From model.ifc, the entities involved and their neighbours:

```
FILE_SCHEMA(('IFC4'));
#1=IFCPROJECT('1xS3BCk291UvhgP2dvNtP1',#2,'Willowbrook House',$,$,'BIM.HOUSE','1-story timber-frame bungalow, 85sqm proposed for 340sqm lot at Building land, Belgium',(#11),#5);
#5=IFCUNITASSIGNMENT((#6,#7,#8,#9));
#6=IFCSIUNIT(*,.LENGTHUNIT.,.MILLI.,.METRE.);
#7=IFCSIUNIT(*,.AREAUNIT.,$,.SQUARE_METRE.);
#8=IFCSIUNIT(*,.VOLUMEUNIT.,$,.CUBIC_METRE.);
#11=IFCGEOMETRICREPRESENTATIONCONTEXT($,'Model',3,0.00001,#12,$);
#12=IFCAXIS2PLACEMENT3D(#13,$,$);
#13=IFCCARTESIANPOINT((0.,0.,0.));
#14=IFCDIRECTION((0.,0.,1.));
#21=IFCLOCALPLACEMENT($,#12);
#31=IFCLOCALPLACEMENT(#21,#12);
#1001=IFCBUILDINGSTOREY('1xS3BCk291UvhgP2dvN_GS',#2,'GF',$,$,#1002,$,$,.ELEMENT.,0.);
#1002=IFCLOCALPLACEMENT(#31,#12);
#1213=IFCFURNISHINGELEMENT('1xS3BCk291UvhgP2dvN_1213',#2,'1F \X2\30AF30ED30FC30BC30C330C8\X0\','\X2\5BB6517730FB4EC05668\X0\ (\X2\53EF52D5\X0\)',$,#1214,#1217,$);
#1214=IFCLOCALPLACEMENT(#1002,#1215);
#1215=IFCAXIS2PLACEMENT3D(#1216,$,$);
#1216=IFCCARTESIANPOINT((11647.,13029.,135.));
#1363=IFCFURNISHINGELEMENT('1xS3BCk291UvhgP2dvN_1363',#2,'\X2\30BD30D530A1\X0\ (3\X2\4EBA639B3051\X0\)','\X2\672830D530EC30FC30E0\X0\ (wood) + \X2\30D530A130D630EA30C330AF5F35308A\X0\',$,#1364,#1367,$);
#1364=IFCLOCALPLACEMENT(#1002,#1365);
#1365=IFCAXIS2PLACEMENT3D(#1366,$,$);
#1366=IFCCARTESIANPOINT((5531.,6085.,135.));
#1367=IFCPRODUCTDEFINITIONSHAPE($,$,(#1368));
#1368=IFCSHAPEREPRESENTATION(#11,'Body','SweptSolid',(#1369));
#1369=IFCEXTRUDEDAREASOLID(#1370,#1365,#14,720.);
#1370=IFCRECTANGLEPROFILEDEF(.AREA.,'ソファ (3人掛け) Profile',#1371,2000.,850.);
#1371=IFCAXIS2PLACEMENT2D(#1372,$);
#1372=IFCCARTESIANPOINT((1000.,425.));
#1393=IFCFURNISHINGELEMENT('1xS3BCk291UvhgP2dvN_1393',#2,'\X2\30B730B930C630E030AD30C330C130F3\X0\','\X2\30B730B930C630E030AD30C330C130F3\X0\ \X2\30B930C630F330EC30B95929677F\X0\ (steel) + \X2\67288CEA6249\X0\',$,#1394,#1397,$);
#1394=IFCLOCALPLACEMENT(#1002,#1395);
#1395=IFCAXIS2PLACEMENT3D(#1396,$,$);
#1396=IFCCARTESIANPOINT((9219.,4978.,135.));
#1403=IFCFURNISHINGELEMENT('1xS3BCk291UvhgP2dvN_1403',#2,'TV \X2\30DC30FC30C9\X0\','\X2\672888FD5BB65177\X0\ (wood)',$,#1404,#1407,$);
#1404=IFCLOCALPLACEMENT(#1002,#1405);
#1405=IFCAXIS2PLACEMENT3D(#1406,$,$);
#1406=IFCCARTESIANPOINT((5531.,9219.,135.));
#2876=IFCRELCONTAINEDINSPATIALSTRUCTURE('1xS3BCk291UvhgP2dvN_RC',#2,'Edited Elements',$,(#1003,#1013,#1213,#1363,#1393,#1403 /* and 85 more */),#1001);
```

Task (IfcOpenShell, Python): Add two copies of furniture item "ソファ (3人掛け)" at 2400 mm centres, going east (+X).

```python
import numpy as np
import ifcopenshell
import ifcopenshell.api.geometry
import ifcopenshell.api.root
import ifcopenshell.util.element
import ifcopenshell.util.placement

model = ifcopenshell.open("model.ifc")


def reuse_history(source, copy):
    """copy_class also copies each property set's owner history, people and application; keep the originals."""
    for rel in copy.IsDefinedBy:
        if rel.is_a("IfcRelDefinesByProperties") and (history := rel.RelatingPropertyDefinition.OwnerHistory):
            rel.RelatingPropertyDefinition.OwnerHistory = source.OwnerHistory
            ifcopenshell.util.element.remove_deep2(model, history)


source = model.by_guid("1xS3BCk291UvhgP2dvN_1363")
base = ifcopenshell.util.placement.get_local_placement(source.ObjectPlacement)
step = np.array([1.0, 0.0, 0.0]) * 2400.0

for i in range(1, 3):
    copy = ifcopenshell.api.root.copy_class(model, product=source)
    copy.Representation = ifcopenshell.util.element.copy_deep(
        model, source.Representation, exclude=["IfcGeometricRepresentationContext", "IfcRepresentationMap"]
    )
    reuse_history(source, copy)
    matrix = base.copy()
    matrix[:3, 3] += i * step
    print("added at", matrix[:3, 3].round(3) + 0.0)
    ifcopenshell.api.geometry.edit_object_placement(model, product=copy, matrix=matrix, is_si=False)

model.write("model_edited.ifc")
```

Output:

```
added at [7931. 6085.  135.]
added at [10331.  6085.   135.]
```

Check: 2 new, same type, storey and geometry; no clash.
